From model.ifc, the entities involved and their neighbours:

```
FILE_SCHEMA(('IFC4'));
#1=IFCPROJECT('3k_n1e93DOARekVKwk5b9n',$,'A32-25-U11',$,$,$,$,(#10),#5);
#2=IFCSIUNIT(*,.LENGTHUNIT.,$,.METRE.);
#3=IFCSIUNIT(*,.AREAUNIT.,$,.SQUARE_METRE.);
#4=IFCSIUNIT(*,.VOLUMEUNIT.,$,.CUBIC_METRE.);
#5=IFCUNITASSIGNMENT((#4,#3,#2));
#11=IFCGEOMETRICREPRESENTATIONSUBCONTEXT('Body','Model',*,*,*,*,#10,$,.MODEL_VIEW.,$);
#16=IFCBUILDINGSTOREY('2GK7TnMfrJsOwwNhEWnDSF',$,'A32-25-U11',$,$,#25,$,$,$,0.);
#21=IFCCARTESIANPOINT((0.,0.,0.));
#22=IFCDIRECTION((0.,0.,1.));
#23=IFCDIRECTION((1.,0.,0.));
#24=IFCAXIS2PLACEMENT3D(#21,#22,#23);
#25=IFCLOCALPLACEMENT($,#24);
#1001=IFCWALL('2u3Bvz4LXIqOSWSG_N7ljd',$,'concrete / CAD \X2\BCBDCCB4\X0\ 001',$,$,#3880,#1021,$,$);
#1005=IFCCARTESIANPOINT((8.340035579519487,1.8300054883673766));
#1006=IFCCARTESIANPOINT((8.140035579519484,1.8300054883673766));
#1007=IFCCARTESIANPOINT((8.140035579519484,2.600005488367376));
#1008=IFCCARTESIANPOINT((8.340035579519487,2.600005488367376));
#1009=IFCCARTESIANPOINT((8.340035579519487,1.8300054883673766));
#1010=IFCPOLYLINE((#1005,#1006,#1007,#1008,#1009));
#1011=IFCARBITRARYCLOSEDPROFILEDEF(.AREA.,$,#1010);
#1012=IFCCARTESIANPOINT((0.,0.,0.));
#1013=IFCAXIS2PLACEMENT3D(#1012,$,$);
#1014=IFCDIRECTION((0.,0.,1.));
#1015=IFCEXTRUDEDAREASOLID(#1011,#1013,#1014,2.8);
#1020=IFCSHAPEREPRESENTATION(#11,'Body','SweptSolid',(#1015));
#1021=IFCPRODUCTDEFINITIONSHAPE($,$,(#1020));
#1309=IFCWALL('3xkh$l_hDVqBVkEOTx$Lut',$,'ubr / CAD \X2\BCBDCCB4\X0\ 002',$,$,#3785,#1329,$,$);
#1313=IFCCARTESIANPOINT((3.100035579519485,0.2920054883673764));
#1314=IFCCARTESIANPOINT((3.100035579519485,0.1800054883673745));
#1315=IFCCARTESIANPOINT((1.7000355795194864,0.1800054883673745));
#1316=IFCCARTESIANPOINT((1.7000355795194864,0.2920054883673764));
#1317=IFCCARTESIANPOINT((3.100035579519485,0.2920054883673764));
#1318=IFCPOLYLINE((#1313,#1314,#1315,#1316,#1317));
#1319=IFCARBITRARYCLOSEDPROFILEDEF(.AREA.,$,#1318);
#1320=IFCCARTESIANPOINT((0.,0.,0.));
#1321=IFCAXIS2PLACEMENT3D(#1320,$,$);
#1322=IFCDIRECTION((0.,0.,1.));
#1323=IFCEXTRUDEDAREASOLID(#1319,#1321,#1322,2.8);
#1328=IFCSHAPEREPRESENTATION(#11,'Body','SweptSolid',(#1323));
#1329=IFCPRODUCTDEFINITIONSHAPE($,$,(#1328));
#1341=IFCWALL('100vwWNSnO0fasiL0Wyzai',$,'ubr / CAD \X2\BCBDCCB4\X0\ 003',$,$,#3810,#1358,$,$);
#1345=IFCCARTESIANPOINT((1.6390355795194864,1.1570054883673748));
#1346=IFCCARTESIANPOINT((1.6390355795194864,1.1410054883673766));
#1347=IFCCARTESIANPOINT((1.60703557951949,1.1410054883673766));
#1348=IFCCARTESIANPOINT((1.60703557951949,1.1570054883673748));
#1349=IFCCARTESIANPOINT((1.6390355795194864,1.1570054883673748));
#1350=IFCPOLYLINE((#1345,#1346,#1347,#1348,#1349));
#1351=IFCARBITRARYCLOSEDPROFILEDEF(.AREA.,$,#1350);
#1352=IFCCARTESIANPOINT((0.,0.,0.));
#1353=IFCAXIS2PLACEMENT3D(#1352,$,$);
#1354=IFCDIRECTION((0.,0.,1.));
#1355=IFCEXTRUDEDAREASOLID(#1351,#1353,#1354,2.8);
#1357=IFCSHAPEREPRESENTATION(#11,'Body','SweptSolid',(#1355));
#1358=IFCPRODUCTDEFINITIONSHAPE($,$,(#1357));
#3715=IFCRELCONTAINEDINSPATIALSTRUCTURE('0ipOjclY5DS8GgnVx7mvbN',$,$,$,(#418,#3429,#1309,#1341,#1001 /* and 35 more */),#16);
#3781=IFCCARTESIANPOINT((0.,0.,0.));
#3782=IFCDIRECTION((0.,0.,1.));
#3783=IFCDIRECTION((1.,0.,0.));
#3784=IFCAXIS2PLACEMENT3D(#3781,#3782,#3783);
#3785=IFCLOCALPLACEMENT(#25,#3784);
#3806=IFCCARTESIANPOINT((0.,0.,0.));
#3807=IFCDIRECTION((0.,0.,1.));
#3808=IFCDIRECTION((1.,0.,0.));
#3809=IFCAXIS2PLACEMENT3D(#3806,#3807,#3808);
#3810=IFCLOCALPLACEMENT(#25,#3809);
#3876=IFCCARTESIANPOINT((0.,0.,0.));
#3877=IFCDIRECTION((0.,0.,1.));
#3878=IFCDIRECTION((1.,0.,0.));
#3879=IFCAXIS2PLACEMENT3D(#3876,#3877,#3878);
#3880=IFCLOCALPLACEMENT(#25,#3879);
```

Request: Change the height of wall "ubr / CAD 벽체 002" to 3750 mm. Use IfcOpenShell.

```python
import ifcopenshell
import ifcopenshell.geom
import ifcopenshell.util.representation
import ifcopenshell.util.shape

model = ifcopenshell.open("model.ifc")
settings = ifcopenshell.geom.settings()


def volume(element):
    """Net volume in cubic metres, openings subtracted."""
    shape = ifcopenshell.geom.create_shape(settings, element)
    return ifcopenshell.util.shape.get_volume(shape.geometry)


wall = model.by_guid("3xkh$l_hDVqBVkEOTx$Lut")
before = volume(wall)

body = ifcopenshell.util.representation.get_representation(wall, "Model", "Body")
solid = body.Items[0]
old_height = solid.Depth
solid.Depth = 3.75
after = volume(wall)

print(f"height {old_height:g} -> {solid.Depth:g}, volume {before:.3f} -> {after:.3f} m3")

model.write("model_rev.ifc")
```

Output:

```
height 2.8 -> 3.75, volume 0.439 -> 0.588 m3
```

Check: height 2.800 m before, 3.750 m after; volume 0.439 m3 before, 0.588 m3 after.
